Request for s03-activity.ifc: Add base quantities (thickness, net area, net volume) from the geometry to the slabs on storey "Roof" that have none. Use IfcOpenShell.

First a look at what the model holds.

```python
import ifcopenshell
import ifcopenshell.util.element
import ifcopenshell.util.unit

model = ifcopenshell.open("s03-activity.ifc")
print(model.schema)
for unit_type in ("LENGTHUNIT", "AREAUNIT", "VOLUMEUNIT"):
    print(unit_type, ifcopenshell.util.unit.calculate_unit_scale(model, unit_type))
storey = next(s for s in model.by_type("IfcBuildingStorey") if s.Name == "Roof")
slabs = [e for e in ifcopenshell.util.element.get_decomposition(storey) if e.is_a("IfcSlab")]
for e in sorted(slabs, key=lambda e: e.id()):
    print(e.id(), e.is_a(), e.Name, list(ifcopenshell.util.element.get_psets(e, qtos_only=True)), sep=" | ")
```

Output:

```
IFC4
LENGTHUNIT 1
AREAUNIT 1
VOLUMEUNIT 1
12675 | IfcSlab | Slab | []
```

```python
import ifcopenshell
import ifcopenshell.api.pset
import ifcopenshell.geom
import ifcopenshell.util.element
import ifcopenshell.util.shape
import ifcopenshell.util.unit

model = ifcopenshell.open("s03-activity.ifc")
unit_scale = ifcopenshell.util.unit.calculate_unit_scale(model)
area_scale = ifcopenshell.util.unit.calculate_unit_scale(model, "AREAUNIT")
volume_scale = ifcopenshell.util.unit.calculate_unit_scale(model, "VOLUMEUNIT")
settings = ifcopenshell.geom.settings()

storey = next(s for s in model.by_type("IfcBuildingStorey") if s.Name == "Roof")
slabs = [e for e in ifcopenshell.util.element.get_decomposition(storey) if e.is_a("IfcSlab")]

for e in sorted(slabs, key=lambda e: e.id()):
    if ifcopenshell.util.element.get_psets(e, qtos_only=True, should_inherit=False):
        continue
    # Geometry comes back in metres, in the element's own axes.
    shape = ifcopenshell.geom.create_shape(settings, e)
    values = {
        "Width": ifcopenshell.util.shape.get_z(shape.geometry) / unit_scale,
        "NetArea": ifcopenshell.util.shape.get_footprint_area(shape.geometry) / area_scale,
        "NetVolume": ifcopenshell.util.shape.get_volume(shape.geometry) / volume_scale,
    }
    qto = ifcopenshell.api.pset.add_qto(model, product=e, name="Qto_SlabBaseQuantities")
    ifcopenshell.api.pset.edit_qto(model, qto=qto, properties=values)
    print(e.id(), {k: round(v, 3) for k, v in values.items()})

model.write("s03-activity_updated.ifc")
```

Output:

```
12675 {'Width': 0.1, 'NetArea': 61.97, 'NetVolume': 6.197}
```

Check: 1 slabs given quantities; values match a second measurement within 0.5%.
